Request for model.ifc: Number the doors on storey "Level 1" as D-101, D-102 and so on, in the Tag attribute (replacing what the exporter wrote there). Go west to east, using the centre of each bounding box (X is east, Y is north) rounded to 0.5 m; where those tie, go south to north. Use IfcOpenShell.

First a look at what the model holds.

```python
import ifcopenshell
import ifcopenshell.util.element
import ifcopenshell.util.placement

model = ifcopenshell.open("model.ifc")
print(model.schema)
storey = next(s for s in model.by_type("IfcBuildingStorey") if s.Name == "Level 1")
doors = [e for e in ifcopenshell.util.element.get_decomposition(storey) if e.is_a("IfcDoor")]
for e in sorted(doors, key=lambda e: e.id()):
    origin = ifcopenshell.util.placement.get_local_placement(e.ObjectPlacement)[:3, 3]
    print(e.id(), e.Tag, e.Name, origin.round(2) + 0.0, sep=" | ")
```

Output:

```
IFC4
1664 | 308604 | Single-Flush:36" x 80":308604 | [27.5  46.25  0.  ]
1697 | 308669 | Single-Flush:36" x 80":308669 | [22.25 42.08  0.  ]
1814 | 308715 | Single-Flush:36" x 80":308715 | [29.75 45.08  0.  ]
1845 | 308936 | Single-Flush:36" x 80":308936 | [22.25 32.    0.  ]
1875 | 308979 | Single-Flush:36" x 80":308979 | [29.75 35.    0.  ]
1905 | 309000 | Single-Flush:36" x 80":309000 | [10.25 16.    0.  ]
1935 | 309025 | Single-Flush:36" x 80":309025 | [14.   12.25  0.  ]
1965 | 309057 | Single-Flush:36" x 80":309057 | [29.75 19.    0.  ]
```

```python
import ifcopenshell
import ifcopenshell.geom
import ifcopenshell.util.element
import ifcopenshell.util.shape

model = ifcopenshell.open("model.ifc")
settings = ifcopenshell.geom.settings()
settings.set("use-world-coords", True)


def centre(element):
    shape = ifcopenshell.geom.create_shape(settings, element)
    return ifcopenshell.util.shape.get_bbox_centroid(shape.geometry)


storey = next(s for s in model.by_type("IfcBuildingStorey") if s.Name == "Level 1")
doors = [e for e in ifcopenshell.util.element.get_decomposition(storey) if e.is_a("IfcDoor")]

# Insertion points can sit at a corner or the storey origin, so sort by the geometry (in metres).
centres = {e: centre(e) for e in doors}
doors.sort(key=lambda e: (round(centres[e][0] / 0.5), centres[e][1]))

for i, e in enumerate(doors, start=1):
    number = f"D-1{i:02d}"
    e.Tag = number
    print(e.id(), number)

model.write("model_v2.ifc")
```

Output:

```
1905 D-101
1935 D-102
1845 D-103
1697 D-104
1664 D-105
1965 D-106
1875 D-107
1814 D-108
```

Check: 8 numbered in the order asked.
